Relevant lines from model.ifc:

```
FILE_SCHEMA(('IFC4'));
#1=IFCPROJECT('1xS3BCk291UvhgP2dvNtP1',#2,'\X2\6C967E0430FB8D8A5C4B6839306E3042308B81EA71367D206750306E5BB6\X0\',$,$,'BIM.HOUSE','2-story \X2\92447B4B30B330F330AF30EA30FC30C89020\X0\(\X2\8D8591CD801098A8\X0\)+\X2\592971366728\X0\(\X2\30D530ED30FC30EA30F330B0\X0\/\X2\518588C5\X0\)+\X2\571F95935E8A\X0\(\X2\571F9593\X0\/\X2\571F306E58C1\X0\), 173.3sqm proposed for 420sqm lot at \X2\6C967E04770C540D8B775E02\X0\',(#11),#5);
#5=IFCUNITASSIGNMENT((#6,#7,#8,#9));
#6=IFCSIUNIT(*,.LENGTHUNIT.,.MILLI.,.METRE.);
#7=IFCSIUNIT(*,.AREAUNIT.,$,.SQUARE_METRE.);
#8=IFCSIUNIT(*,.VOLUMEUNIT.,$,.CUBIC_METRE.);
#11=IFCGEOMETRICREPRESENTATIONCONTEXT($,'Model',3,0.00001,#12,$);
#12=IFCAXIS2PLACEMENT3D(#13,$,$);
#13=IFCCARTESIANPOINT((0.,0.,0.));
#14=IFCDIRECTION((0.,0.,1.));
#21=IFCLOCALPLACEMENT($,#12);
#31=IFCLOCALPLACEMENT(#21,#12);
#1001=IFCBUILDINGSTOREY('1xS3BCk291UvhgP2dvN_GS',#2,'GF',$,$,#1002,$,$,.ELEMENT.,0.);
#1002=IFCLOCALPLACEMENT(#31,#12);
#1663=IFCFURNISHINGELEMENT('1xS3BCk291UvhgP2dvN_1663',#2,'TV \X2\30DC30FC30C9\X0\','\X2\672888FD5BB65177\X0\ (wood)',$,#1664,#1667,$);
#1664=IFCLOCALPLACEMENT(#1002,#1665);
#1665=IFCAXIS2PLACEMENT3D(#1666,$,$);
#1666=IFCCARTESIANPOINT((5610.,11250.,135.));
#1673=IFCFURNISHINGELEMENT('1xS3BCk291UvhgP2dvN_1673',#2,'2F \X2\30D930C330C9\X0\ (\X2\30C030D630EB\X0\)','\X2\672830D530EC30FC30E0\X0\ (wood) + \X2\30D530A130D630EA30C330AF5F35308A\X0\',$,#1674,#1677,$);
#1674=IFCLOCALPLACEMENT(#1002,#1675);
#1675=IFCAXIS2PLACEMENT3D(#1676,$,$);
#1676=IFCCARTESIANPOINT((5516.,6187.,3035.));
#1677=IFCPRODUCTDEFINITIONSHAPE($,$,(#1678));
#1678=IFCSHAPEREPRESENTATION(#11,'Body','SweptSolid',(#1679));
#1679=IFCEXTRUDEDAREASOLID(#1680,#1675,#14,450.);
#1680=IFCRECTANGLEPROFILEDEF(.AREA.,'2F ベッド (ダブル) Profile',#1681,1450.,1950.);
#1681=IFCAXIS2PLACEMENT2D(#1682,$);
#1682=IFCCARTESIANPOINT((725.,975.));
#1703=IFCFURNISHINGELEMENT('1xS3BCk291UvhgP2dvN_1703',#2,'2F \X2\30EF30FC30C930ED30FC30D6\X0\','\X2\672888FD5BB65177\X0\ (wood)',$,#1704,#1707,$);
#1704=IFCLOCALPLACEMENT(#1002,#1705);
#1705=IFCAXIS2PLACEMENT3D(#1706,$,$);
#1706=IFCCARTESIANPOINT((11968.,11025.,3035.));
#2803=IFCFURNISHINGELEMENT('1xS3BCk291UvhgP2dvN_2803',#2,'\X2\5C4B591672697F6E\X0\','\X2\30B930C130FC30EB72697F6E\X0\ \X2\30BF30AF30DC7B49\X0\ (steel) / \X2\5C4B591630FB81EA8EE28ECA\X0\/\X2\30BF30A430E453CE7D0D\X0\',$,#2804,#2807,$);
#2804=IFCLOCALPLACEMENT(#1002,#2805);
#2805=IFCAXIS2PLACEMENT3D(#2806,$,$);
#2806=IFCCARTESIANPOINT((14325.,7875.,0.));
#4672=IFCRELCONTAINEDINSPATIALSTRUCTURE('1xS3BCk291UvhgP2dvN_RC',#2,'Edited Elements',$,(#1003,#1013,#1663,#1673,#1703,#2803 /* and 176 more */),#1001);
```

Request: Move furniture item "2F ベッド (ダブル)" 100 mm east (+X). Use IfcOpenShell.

```python
import ifcopenshell
import ifcopenshell.api.geometry
import ifcopenshell.util.placement

model = ifcopenshell.open("model.ifc")

item = model.by_id(1673)
matrix = ifcopenshell.util.placement.get_local_placement(item.ObjectPlacement)
matrix[0, 3] += 100.0
ifcopenshell.api.geometry.edit_object_placement(model, product=item, matrix=matrix, is_si=False)

print(ifcopenshell.util.placement.get_local_placement(item.ObjectPlacement).round(3) + 0.0)

model.write("model_v2.ifc")
```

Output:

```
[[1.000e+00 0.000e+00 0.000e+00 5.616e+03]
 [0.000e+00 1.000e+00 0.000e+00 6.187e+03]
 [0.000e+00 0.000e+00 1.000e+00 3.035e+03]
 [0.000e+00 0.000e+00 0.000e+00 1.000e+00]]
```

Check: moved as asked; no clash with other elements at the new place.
